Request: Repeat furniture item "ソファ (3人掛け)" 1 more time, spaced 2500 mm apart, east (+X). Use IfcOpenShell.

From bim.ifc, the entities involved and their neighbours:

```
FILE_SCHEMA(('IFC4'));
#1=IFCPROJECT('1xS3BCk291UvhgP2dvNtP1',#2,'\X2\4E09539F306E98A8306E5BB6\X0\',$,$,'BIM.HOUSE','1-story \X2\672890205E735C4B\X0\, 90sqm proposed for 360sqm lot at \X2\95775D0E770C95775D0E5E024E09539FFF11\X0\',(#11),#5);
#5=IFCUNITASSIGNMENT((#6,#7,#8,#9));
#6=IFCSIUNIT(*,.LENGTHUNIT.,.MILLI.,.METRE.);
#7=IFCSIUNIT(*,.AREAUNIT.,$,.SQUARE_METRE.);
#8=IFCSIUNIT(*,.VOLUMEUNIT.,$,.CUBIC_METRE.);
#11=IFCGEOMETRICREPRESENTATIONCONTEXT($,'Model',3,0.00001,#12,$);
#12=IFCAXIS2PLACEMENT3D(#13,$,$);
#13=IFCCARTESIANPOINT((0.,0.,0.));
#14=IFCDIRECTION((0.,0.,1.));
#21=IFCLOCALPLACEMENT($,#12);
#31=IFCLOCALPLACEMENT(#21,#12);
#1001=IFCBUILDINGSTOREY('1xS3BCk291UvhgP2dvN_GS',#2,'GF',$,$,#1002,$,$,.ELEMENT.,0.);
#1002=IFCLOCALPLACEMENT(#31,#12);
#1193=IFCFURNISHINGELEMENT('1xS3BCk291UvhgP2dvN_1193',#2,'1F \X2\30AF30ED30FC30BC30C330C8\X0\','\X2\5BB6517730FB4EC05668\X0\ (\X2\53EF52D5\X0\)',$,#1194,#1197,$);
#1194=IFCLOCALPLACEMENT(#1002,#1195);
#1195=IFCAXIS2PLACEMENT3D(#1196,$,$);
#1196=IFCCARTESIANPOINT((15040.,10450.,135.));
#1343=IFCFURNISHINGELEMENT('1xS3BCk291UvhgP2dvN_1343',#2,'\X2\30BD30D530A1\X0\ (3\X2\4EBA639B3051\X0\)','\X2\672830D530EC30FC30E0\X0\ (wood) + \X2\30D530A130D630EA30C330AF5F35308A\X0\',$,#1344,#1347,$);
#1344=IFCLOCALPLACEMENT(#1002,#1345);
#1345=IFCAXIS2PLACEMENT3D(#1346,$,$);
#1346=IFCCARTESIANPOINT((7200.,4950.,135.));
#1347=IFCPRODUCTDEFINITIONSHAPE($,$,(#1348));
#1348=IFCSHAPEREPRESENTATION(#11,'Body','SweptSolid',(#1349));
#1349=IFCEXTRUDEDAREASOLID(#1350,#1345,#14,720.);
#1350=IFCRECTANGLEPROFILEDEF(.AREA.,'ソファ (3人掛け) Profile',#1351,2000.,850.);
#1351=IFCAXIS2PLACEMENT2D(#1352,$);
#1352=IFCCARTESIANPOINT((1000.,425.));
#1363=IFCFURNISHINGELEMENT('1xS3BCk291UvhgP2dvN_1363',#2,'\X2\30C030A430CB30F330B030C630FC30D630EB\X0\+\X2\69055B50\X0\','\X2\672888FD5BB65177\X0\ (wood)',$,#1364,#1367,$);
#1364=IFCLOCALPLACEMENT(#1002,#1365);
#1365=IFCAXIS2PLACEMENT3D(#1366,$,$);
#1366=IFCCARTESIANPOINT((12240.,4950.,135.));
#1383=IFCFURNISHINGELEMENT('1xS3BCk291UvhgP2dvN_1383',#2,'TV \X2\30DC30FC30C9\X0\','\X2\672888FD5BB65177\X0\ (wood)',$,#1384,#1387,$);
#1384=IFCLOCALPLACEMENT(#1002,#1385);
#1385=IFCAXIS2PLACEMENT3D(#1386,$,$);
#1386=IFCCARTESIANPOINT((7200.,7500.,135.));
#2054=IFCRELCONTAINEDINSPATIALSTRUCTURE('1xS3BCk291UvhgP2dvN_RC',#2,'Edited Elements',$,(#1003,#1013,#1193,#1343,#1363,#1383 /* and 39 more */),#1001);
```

```python
import numpy as np
import ifcopenshell
import ifcopenshell.api.geometry
import ifcopenshell.api.root
import ifcopenshell.util.element
import ifcopenshell.util.placement
import ifcopenshell.util.unit

model = ifcopenshell.open("bim.ifc")
unit_scale = ifcopenshell.util.unit.calculate_unit_scale(model)


def reuse_history(source, copy):
    """copy_class also copies each property set's owner history, people and application; keep the originals."""
    for rel in copy.IsDefinedBy:
        if rel.is_a("IfcRelDefinesByProperties") and (history := rel.RelatingPropertyDefinition.OwnerHistory):
            rel.RelatingPropertyDefinition.OwnerHistory = source.OwnerHistory
            ifcopenshell.util.element.remove_deep2(model, history)


source = model.by_guid("1xS3BCk291UvhgP2dvN_1343")
base = ifcopenshell.util.placement.get_local_placement(source.ObjectPlacement)
step = np.array([1.0, 0.0, 0.0]) * 2.5 / unit_scale

for i in range(1, 2):
    copy = ifcopenshell.api.root.copy_class(model, product=source)
    copy.Representation = ifcopenshell.util.element.copy_deep(
        model, source.Representation, exclude=["IfcGeometricRepresentationContext", "IfcRepresentationMap"]
    )
    reuse_history(source, copy)
    matrix = base.copy()
    matrix[:3, 3] += i * step
    print("added at", matrix[:3, 3].round(3) + 0.0)
    ifcopenshell.api.geometry.edit_object_placement(model, product=copy, matrix=matrix, is_si=False)

model.write("bim_updated.ifc")
```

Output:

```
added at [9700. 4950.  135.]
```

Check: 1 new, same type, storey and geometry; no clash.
